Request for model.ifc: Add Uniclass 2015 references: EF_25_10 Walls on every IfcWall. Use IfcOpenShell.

First a look at what the model holds.

```python
import ifcopenshell

model = ifcopenshell.open("model.ifc")
print(model.schema)
print("classifications:", [c.Name for c in model.by_type("IfcClassification")])
for ifc_class in ("IfcDoor", "IfcRoof", "IfcStair", "IfcWall", "IfcWindow"):
    print(ifc_class, len(model.by_type(ifc_class)))
```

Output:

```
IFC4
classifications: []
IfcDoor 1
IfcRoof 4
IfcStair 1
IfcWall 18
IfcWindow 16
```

```python
import ifcopenshell
import ifcopenshell.api.classification

model = ifcopenshell.open("model.ifc")

system = ifcopenshell.api.classification.add_classification(model, classification="Uniclass 2015")

codes = {
    "IfcWall": ("EF_25_10", "Walls"),
}
for ifc_class, (code, name) in codes.items():
    products = model.by_type(ifc_class)
    ifcopenshell.api.classification.add_reference(
        model, products=products, classification=system, identification=code, name=name
    )
    print(code, len(products))

model.write("model_rev.ifc")
```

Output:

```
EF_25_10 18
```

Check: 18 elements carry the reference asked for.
